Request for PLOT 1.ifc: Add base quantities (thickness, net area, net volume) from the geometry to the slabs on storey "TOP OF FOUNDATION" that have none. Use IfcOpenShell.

First a look at what the model holds.

```python
import ifcopenshell
import ifcopenshell.util.element
import ifcopenshell.util.unit

model = ifcopenshell.open("PLOT 1.ifc")
print(model.schema)
for unit_type in ("LENGTHUNIT", "AREAUNIT", "VOLUMEUNIT"):
    print(unit_type, ifcopenshell.util.unit.calculate_unit_scale(model, unit_type))
storey = next(s for s in model.by_type("IfcBuildingStorey") if s.Name == "TOP OF FOUNDATION")
slabs = [e for e in ifcopenshell.util.element.get_decomposition(storey) if e.is_a("IfcSlab")]
for e in sorted(slabs, key=lambda e: e.id()):
    print(e.id(), e.is_a(), e.Name, list(ifcopenshell.util.element.get_psets(e, qtos_only=True)), sep=" | ")
```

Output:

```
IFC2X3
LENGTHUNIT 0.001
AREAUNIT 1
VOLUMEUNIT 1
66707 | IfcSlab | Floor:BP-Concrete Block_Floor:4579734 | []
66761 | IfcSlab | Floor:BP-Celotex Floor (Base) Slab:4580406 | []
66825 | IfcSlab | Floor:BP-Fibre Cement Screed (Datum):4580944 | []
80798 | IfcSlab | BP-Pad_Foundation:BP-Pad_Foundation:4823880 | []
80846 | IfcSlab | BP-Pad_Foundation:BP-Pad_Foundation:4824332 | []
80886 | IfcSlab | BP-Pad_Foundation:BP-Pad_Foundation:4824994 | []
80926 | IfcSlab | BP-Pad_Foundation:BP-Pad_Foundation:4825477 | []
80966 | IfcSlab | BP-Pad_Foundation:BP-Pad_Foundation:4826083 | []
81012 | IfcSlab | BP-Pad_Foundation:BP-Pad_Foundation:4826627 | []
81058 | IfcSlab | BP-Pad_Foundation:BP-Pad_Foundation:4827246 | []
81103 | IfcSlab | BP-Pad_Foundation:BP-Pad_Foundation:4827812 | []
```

```python
import ifcopenshell
import ifcopenshell.api.pset
import ifcopenshell.geom
import ifcopenshell.util.element
import ifcopenshell.util.shape
import ifcopenshell.util.unit

model = ifcopenshell.open("PLOT 1.ifc")
unit_scale = ifcopenshell.util.unit.calculate_unit_scale(model)
area_scale = ifcopenshell.util.unit.calculate_unit_scale(model, "AREAUNIT")
volume_scale = ifcopenshell.util.unit.calculate_unit_scale(model, "VOLUMEUNIT")
settings = ifcopenshell.geom.settings()

storey = next(s for s in model.by_type("IfcBuildingStorey") if s.Name == "TOP OF FOUNDATION")
slabs = [e for e in ifcopenshell.util.element.get_decomposition(storey) if e.is_a("IfcSlab")]

for e in sorted(slabs, key=lambda e: e.id()):
    if ifcopenshell.util.element.get_psets(e, qtos_only=True, should_inherit=False):
        continue
    # Geometry comes back in metres, in the element's own axes.
    shape = ifcopenshell.geom.create_shape(settings, e)
    values = {
        "Width": ifcopenshell.util.shape.get_z(shape.geometry) / unit_scale,
        "NetArea": ifcopenshell.util.shape.get_footprint_area(shape.geometry) / area_scale,
        "NetVolume": ifcopenshell.util.shape.get_volume(shape.geometry) / volume_scale,
    }
    qto = ifcopenshell.api.pset.add_qto(model, product=e, name="BaseQuantities")
    ifcopenshell.api.pset.edit_qto(model, qto=qto, properties=values)
    print(e.id(), {k: round(v, 3) for k, v in values.items()})

model.write("PLOT 1_rev.ifc")
```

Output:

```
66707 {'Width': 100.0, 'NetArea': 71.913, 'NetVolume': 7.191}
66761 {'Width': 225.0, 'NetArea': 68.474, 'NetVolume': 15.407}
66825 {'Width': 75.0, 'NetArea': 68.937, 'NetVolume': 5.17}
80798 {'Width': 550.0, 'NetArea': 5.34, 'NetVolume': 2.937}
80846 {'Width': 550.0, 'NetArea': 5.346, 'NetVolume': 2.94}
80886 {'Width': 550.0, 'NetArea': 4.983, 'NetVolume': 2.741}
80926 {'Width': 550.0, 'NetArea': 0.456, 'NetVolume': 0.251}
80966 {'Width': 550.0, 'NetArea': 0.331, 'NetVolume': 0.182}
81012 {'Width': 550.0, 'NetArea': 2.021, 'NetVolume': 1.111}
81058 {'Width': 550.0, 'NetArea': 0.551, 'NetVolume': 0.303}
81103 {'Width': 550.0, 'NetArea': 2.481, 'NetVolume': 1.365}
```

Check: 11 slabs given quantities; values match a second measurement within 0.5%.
